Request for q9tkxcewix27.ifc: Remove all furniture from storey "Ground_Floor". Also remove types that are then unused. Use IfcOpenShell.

First a look at what the model holds.

```python
import ifcopenshell
import ifcopenshell.util.element

model = ifcopenshell.open("q9tkxcewix27.ifc")
print(model.schema)
storey = next(s for s in model.by_type("IfcBuildingStorey") if s.Name == "Ground_Floor")
furniture = [e for e in ifcopenshell.util.element.get_decomposition(storey) if e.is_a("IfcFurnishingElement")]
seen = {}
for e in furniture:
    element_type = ifcopenshell.util.element.get_type(e)
    name = element_type.Name if element_type not in (None, e) else None
    seen[name] = seen.get(name, 0) + 1
for name, count in sorted(seen.items(), key=str):
    print(count, "x", name)
```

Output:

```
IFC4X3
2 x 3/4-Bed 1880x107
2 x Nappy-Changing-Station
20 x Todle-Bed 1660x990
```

```python
import ifcopenshell
import ifcopenshell.api.root
import ifcopenshell.util.element

model = ifcopenshell.open("q9tkxcewix27.ifc")

storey = next(s for s in model.by_type("IfcBuildingStorey") if s.Name == "Ground_Floor")
furniture = [e for e in ifcopenshell.util.element.get_decomposition(storey) if e.is_a("IfcFurnishingElement")]
types = {ifcopenshell.util.element.get_type(e) for e in furniture} - {None, *furniture}

for e in furniture:
    ifcopenshell.api.root.remove_product(model, product=e)
print(len(furniture), "removed")

unused = [t for t in types if not ifcopenshell.util.element.get_types(t)]
for t in unused:
    ifcopenshell.api.root.remove_product(model, product=t)
print(len(unused), "unused types removed")

model.write("q9tkxcewix27_v2.ifc")
```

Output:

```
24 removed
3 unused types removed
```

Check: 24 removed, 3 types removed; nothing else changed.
